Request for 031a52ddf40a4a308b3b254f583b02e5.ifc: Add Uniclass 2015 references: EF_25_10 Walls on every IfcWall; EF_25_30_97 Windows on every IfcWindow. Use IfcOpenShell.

First a look at what the model holds.

```python
import ifcopenshell

model = ifcopenshell.open("031a52ddf40a4a308b3b254f583b02e5.ifc")
print(model.schema)
print("classifications:", [c.Name for c in model.by_type("IfcClassification")])
for ifc_class in ("IfcDoor", "IfcRoof", "IfcStair", "IfcWall", "IfcWindow"):
    print(ifc_class, len(model.by_type(ifc_class)))
```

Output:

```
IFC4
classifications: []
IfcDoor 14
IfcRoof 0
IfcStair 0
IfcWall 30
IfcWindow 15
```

```python
import ifcopenshell
import ifcopenshell.api.classification

model = ifcopenshell.open("031a52ddf40a4a308b3b254f583b02e5.ifc")

system = ifcopenshell.api.classification.add_classification(model, classification="Uniclass 2015")

codes = {
    "IfcWall": ("EF_25_10", "Walls"),
    "IfcWindow": ("EF_25_30_97", "Windows"),
}
for ifc_class, (code, name) in codes.items():
    products = model.by_type(ifc_class)
    ifcopenshell.api.classification.add_reference(
        model, products=products, classification=system, identification=code, name=name
    )
    print(code, len(products))

model.write("031a52ddf40a4a308b3b254f583b02e5_v2.ifc")
```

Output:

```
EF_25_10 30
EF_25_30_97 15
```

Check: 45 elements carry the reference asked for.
